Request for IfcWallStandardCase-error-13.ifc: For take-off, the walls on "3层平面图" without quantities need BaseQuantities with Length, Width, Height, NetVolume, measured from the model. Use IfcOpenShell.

First a look at what the model holds.

```python
import ifcopenshell
import ifcopenshell.util.element
import ifcopenshell.util.unit

model = ifcopenshell.open("IfcWallStandardCase-error-13.ifc")
print(model.schema)
for unit_type in ("LENGTHUNIT", "AREAUNIT", "VOLUMEUNIT"):
    print(unit_type, ifcopenshell.util.unit.calculate_unit_scale(model, unit_type))
storey = next(s for s in model.by_type("IfcBuildingStorey") if s.Name == "3层平面图")
walls = [e for e in ifcopenshell.util.element.get_decomposition(storey) if e.is_a("IfcWall")]
for e in sorted(walls, key=lambda e: e.id()):
    print(e.id(), e.is_a(), e.Name, list(ifcopenshell.util.element.get_psets(e, qtos_only=True)), sep=" | ")
```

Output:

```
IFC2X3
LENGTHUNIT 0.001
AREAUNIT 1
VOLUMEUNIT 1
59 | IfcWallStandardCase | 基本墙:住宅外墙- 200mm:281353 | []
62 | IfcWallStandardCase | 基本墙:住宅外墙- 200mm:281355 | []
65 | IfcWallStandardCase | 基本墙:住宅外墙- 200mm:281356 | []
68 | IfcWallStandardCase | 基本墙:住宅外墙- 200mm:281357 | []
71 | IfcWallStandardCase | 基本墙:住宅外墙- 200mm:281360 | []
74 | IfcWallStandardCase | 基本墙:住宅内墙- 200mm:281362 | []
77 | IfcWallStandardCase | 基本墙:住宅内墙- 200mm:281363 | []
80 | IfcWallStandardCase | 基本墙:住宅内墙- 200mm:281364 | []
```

```python
import ifcopenshell
import ifcopenshell.api.pset
import ifcopenshell.geom
import ifcopenshell.util.element
import ifcopenshell.util.shape
import ifcopenshell.util.unit

model = ifcopenshell.open("IfcWallStandardCase-error-13.ifc")
unit_scale = ifcopenshell.util.unit.calculate_unit_scale(model)
volume_scale = ifcopenshell.util.unit.calculate_unit_scale(model, "VOLUMEUNIT")
settings = ifcopenshell.geom.settings()

storey = next(s for s in model.by_type("IfcBuildingStorey") if s.Name == "3层平面图")
walls = [e for e in ifcopenshell.util.element.get_decomposition(storey) if e.is_a("IfcWall")]

for e in sorted(walls, key=lambda e: e.id()):
    if ifcopenshell.util.element.get_psets(e, qtos_only=True, should_inherit=False):
        continue
    # Geometry comes back in metres, in the element's own axes.
    shape = ifcopenshell.geom.create_shape(settings, e)
    values = {
        "Length": ifcopenshell.util.shape.get_x(shape.geometry) / unit_scale,
        "Width": ifcopenshell.util.shape.get_y(shape.geometry) / unit_scale,
        "Height": ifcopenshell.util.shape.get_z(shape.geometry) / unit_scale,
        "NetVolume": ifcopenshell.util.shape.get_volume(shape.geometry) / volume_scale,
    }
    qto = ifcopenshell.api.pset.add_qto(model, product=e, name="BaseQuantities")
    ifcopenshell.api.pset.edit_qto(model, qto=qto, properties=values)
    print(e.id(), {k: round(v, 3) for k, v in values.items()})

model.write("IfcWallStandardCase-error-13_rev.ifc")
```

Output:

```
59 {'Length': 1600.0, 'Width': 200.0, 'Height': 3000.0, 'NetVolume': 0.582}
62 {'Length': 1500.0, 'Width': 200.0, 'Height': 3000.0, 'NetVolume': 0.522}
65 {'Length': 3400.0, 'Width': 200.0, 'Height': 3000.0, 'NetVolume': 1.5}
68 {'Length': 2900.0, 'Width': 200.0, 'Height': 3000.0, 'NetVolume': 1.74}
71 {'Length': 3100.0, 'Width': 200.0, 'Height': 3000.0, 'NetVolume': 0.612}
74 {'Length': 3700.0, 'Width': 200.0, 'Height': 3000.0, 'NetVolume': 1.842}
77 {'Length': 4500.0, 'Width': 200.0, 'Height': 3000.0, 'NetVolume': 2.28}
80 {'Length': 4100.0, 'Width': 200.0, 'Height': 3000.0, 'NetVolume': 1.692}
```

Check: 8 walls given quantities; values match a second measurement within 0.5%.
